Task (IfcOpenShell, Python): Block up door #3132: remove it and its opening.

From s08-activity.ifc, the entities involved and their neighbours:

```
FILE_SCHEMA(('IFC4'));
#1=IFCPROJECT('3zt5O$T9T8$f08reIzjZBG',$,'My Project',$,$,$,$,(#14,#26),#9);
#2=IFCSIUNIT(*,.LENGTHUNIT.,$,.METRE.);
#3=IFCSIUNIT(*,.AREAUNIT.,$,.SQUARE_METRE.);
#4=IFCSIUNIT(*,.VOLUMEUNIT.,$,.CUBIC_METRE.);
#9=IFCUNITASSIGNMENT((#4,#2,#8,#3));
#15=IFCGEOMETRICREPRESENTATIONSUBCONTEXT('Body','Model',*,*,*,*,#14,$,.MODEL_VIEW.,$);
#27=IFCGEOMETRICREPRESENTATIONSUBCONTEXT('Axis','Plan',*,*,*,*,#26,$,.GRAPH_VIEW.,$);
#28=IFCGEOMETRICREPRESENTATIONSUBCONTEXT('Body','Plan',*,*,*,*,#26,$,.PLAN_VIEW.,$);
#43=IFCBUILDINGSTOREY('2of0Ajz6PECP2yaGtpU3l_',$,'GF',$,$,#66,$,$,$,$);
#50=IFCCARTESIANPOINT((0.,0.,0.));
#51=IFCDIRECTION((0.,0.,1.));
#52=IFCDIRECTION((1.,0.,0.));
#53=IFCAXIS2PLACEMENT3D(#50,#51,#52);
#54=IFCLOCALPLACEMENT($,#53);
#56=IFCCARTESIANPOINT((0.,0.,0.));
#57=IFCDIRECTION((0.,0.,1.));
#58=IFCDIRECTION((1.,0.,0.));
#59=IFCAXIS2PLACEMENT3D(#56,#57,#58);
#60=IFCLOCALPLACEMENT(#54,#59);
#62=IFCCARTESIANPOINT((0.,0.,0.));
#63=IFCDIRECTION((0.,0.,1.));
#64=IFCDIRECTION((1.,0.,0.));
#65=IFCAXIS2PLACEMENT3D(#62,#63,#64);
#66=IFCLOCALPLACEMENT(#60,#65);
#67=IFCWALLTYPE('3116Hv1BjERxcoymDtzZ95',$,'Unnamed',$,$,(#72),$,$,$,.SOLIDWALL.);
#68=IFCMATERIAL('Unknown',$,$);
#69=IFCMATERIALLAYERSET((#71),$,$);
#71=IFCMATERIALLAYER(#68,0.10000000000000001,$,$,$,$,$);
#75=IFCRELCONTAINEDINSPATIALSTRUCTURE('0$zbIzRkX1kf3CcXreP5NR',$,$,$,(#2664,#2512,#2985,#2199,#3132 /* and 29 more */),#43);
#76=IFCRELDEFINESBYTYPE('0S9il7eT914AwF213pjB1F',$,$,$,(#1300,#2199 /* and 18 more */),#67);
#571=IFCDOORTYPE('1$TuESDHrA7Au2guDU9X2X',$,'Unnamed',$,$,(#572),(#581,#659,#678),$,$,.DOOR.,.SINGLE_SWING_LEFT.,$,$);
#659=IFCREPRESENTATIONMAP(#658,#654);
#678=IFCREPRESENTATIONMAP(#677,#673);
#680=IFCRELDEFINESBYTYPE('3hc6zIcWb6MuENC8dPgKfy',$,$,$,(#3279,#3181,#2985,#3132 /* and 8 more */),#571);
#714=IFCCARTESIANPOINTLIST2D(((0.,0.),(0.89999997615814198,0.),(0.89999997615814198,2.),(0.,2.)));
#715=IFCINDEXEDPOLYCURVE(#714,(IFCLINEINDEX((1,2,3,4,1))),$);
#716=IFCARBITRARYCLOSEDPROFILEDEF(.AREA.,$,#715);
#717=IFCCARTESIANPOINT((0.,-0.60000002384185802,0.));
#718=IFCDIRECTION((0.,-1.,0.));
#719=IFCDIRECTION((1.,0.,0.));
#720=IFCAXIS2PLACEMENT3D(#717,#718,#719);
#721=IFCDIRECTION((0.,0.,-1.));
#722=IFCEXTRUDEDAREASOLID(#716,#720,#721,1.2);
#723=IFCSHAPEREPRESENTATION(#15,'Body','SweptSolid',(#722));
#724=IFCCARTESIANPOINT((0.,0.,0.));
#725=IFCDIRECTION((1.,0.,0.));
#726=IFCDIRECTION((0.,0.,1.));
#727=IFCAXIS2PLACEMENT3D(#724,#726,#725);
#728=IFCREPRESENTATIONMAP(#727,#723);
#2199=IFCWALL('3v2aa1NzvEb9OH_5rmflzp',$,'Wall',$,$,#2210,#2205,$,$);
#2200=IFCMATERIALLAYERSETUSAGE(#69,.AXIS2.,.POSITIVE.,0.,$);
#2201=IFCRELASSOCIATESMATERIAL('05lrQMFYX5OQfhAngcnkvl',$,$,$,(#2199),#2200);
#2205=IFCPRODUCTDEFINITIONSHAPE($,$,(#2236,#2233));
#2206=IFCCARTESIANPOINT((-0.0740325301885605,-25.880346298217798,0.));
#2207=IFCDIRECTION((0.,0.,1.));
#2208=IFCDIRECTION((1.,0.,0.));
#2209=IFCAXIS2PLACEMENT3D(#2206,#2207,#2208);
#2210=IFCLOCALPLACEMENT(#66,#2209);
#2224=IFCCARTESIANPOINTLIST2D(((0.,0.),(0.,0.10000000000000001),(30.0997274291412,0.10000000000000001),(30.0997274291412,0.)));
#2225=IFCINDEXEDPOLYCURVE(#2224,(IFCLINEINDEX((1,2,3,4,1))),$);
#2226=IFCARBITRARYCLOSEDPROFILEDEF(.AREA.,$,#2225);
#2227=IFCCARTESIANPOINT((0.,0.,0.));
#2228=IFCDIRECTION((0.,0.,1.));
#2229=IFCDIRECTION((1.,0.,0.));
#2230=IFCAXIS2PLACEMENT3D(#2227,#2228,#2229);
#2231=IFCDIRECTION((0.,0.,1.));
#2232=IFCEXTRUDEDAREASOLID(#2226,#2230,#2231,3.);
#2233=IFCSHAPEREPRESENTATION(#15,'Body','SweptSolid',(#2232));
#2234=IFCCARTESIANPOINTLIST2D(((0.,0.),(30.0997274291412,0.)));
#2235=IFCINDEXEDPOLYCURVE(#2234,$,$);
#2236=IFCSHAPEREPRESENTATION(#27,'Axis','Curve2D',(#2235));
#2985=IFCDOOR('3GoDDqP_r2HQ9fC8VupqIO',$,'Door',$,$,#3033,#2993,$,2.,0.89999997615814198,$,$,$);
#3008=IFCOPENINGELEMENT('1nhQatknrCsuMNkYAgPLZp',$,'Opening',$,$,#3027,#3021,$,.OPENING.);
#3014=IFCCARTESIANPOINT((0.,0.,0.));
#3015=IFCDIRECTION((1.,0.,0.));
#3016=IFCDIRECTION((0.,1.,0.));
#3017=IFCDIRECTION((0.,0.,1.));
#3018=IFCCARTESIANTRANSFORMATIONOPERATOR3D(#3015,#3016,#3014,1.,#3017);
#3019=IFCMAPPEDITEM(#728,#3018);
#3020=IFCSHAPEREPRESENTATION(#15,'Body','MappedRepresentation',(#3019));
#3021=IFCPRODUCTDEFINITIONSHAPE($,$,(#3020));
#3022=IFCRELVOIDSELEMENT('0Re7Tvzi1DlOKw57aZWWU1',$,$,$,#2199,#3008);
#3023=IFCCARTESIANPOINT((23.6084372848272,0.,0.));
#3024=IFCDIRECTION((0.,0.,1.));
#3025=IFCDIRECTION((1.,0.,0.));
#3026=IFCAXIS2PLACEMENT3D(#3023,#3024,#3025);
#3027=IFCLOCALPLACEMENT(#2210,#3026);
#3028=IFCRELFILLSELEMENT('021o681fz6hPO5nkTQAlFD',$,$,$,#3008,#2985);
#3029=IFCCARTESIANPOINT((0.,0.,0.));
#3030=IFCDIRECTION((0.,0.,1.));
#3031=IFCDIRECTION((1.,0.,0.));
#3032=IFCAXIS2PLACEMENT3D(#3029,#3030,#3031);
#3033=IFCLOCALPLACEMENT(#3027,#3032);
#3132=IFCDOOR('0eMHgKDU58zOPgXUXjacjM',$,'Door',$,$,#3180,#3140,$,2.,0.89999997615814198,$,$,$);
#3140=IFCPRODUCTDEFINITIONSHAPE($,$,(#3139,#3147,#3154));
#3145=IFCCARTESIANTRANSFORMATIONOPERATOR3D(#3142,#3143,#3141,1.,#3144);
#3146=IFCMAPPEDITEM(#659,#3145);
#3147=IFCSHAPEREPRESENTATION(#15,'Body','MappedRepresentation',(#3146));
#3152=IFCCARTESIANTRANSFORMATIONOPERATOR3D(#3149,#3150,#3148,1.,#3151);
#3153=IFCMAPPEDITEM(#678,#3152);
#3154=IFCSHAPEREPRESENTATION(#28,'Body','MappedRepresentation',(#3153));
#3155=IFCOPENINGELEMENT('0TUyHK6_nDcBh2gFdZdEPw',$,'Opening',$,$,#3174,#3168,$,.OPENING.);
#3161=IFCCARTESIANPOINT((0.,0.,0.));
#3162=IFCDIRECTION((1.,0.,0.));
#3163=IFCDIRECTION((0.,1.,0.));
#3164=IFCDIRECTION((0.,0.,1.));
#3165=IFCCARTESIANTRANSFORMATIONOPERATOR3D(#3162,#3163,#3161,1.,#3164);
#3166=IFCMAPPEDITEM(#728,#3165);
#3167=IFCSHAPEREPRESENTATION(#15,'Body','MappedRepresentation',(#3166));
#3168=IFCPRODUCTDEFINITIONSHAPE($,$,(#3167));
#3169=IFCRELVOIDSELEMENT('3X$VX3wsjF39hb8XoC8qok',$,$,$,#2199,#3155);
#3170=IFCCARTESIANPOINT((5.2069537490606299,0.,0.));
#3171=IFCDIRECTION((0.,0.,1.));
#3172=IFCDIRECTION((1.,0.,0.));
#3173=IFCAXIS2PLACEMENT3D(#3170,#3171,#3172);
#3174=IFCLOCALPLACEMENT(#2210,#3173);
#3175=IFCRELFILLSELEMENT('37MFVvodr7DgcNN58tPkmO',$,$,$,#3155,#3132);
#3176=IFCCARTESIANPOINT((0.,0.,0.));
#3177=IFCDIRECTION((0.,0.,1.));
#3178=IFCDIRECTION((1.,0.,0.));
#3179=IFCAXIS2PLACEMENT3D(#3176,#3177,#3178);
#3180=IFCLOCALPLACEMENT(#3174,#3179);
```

```python
import ifcopenshell
import ifcopenshell.api.feature
import ifcopenshell.api.root
import ifcopenshell.geom
import ifcopenshell.util.shape

model = ifcopenshell.open("s08-activity.ifc")
settings = ifcopenshell.geom.settings()


def volume(element):
    """Net volume in cubic metres, openings subtracted."""
    shape = ifcopenshell.geom.create_shape(settings, element)
    return ifcopenshell.util.shape.get_volume(shape.geometry)


door = model.by_id(3132)
opening = door.FillsVoids[0].RelatingOpeningElement
wall = opening.VoidsElements[0].RelatingBuildingElement
before = volume(wall)

ifcopenshell.api.root.remove_product(model, product=door)
ifcopenshell.api.feature.remove_feature(model, feature=opening)

after = volume(wall)

print(f"wall volume {before:.3f} -> {after:.3f} m3")

model.write("s08-activity-out.ifc")
```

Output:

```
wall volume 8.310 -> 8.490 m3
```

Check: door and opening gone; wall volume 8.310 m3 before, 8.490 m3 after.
